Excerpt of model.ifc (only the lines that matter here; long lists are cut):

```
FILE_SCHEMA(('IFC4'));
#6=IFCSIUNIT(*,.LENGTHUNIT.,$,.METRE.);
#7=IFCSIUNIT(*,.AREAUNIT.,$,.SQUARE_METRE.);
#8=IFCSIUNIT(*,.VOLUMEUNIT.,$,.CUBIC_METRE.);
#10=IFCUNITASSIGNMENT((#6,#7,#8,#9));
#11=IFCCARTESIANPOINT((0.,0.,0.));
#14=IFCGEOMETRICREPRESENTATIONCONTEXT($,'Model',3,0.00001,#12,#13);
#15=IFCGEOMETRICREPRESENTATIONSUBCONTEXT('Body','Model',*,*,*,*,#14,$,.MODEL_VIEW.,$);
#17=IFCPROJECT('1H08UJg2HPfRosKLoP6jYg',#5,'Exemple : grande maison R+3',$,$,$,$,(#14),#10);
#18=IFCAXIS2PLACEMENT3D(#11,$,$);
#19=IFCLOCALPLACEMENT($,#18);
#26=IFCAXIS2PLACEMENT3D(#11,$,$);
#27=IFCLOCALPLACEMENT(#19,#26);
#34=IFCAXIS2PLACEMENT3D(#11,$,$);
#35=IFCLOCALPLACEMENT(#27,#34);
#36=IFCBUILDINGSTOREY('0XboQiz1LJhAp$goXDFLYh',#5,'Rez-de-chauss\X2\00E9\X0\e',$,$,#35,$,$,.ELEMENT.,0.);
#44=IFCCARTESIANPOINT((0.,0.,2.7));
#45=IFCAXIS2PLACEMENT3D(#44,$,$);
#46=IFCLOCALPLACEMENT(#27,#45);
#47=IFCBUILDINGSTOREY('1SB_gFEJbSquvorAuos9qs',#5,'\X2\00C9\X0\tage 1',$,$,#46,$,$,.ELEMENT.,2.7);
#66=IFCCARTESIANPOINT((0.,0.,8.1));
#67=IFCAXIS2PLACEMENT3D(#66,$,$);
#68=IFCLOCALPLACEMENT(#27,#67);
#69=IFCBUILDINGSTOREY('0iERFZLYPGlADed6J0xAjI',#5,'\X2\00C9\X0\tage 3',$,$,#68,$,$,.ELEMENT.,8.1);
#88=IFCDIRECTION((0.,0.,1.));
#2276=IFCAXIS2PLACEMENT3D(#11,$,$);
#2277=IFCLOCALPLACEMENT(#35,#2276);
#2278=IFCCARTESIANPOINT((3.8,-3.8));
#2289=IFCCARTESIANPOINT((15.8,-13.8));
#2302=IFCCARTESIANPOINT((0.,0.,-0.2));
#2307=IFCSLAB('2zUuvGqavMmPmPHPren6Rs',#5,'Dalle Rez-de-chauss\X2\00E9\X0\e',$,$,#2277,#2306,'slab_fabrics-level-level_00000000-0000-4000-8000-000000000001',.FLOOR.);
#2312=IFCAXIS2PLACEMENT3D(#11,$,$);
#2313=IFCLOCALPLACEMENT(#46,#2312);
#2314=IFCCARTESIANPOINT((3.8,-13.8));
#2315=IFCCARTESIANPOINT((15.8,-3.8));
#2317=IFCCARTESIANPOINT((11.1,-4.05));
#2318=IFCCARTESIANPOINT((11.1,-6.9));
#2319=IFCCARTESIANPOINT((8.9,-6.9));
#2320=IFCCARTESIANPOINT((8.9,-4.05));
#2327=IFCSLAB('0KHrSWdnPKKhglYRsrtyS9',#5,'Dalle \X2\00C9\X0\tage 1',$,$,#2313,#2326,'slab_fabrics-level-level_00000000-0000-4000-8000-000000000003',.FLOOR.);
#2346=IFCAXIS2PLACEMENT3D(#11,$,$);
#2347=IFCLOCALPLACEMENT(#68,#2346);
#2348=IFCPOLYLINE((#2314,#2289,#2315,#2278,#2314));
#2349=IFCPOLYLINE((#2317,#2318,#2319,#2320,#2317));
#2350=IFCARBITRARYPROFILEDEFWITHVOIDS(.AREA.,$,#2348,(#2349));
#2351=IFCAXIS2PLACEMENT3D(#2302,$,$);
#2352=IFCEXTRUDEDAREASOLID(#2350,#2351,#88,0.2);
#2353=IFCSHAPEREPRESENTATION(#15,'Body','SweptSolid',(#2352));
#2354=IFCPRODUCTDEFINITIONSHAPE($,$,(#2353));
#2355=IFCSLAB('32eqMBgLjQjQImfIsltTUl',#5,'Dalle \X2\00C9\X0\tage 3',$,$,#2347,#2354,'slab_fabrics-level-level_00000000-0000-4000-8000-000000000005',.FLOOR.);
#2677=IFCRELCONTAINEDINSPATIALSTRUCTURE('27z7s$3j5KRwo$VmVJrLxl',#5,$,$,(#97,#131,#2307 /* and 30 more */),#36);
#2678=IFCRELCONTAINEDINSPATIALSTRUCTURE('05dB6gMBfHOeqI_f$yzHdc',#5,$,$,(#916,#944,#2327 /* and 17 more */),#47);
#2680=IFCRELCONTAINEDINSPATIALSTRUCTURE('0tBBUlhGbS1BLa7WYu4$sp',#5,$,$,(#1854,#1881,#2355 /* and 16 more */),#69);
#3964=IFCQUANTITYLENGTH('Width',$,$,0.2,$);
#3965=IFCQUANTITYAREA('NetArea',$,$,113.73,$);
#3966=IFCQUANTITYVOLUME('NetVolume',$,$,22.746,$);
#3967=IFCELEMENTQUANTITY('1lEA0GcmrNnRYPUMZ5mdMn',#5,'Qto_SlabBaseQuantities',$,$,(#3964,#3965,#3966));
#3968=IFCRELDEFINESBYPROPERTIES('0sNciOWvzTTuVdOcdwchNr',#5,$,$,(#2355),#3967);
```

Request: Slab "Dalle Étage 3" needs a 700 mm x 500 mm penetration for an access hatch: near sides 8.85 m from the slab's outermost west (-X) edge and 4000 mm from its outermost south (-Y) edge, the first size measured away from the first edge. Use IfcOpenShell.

```python
import numpy as np
import ifcopenshell
import ifcopenshell.api.feature
import ifcopenshell.api.geometry
import ifcopenshell.api.pset
import ifcopenshell.api.root
import ifcopenshell.geom
import ifcopenshell.util.element
import ifcopenshell.util.placement
import ifcopenshell.util.representation
import ifcopenshell.util.shape
import ifcopenshell.util.unit

model = ifcopenshell.open("model.ifc")
unit_scale = ifcopenshell.util.unit.calculate_unit_scale(model)
area_scale = ifcopenshell.util.unit.calculate_unit_scale(model, "AREAUNIT")
volume_scale = ifcopenshell.util.unit.calculate_unit_scale(model, "VOLUMEUNIT")
settings = ifcopenshell.geom.settings()


def volume(element):
    """Net volume in cubic metres, openings subtracted."""
    shape = ifcopenshell.geom.create_shape(settings, element)
    return ifcopenshell.util.shape.get_volume(shape.geometry)


slab = model.by_id(2355)
before = volume(slab)

# Extent in the slab's own axes, in metres. The edges named are its -X and -Y sides.
slab_shape = ifcopenshell.geom.create_shape(settings, slab)
vertices = ifcopenshell.util.shape.get_vertices(slab_shape.geometry)
x_min, y_min, bottom = vertices.min(axis=0)
top = vertices[:, 2].max()

opening = ifcopenshell.api.root.create_entity(model, ifc_class="IfcOpeningElement", name="Access hatch opening", predefined_type="OPENING")
context = ifcopenshell.util.representation.get_context(model, "Model", "Body", "MODEL_VIEW")
width, depth = 0.7, 0.5
outline = [(0.0, 0.0), (width, 0.0), (width, depth), (0.0, depth), (0.0, 0.0)]
# Overshoot both faces by 50 mm so the cut is clean.
shape = ifcopenshell.api.geometry.add_slab_representation(
    model, context=context, depth=top - bottom + 0.1, polyline=outline
)
ifcopenshell.api.geometry.assign_representation(model, product=opening, representation=shape)

matrix = ifcopenshell.util.placement.get_local_placement(slab.ObjectPlacement)
matrix[:, 3] = matrix @ np.append(np.array([x_min + 8.85, y_min + 4, bottom - 0.05]) / unit_scale, 1.0)
ifcopenshell.api.geometry.edit_object_placement(model, product=opening, matrix=matrix, is_si=False)
ifcopenshell.api.feature.add_feature(model, feature=opening, element=slab)

after = volume(slab)

# Update the slab's stored quantities.
qto = model.by_id(ifcopenshell.util.element.get_pset(slab, "Qto_SlabBaseQuantities", should_inherit=False)["id"])
ifcopenshell.api.pset.edit_qto(model, qto=qto, properties={
    "NetArea": after / (top - bottom) / area_scale,
    "NetVolume": after / volume_scale,
})

print(f"slab volume {before:.3f} -> {after:.3f} m3")

model.write("model_edited.ifc")
```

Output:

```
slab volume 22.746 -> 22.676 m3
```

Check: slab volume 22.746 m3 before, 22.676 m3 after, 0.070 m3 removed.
